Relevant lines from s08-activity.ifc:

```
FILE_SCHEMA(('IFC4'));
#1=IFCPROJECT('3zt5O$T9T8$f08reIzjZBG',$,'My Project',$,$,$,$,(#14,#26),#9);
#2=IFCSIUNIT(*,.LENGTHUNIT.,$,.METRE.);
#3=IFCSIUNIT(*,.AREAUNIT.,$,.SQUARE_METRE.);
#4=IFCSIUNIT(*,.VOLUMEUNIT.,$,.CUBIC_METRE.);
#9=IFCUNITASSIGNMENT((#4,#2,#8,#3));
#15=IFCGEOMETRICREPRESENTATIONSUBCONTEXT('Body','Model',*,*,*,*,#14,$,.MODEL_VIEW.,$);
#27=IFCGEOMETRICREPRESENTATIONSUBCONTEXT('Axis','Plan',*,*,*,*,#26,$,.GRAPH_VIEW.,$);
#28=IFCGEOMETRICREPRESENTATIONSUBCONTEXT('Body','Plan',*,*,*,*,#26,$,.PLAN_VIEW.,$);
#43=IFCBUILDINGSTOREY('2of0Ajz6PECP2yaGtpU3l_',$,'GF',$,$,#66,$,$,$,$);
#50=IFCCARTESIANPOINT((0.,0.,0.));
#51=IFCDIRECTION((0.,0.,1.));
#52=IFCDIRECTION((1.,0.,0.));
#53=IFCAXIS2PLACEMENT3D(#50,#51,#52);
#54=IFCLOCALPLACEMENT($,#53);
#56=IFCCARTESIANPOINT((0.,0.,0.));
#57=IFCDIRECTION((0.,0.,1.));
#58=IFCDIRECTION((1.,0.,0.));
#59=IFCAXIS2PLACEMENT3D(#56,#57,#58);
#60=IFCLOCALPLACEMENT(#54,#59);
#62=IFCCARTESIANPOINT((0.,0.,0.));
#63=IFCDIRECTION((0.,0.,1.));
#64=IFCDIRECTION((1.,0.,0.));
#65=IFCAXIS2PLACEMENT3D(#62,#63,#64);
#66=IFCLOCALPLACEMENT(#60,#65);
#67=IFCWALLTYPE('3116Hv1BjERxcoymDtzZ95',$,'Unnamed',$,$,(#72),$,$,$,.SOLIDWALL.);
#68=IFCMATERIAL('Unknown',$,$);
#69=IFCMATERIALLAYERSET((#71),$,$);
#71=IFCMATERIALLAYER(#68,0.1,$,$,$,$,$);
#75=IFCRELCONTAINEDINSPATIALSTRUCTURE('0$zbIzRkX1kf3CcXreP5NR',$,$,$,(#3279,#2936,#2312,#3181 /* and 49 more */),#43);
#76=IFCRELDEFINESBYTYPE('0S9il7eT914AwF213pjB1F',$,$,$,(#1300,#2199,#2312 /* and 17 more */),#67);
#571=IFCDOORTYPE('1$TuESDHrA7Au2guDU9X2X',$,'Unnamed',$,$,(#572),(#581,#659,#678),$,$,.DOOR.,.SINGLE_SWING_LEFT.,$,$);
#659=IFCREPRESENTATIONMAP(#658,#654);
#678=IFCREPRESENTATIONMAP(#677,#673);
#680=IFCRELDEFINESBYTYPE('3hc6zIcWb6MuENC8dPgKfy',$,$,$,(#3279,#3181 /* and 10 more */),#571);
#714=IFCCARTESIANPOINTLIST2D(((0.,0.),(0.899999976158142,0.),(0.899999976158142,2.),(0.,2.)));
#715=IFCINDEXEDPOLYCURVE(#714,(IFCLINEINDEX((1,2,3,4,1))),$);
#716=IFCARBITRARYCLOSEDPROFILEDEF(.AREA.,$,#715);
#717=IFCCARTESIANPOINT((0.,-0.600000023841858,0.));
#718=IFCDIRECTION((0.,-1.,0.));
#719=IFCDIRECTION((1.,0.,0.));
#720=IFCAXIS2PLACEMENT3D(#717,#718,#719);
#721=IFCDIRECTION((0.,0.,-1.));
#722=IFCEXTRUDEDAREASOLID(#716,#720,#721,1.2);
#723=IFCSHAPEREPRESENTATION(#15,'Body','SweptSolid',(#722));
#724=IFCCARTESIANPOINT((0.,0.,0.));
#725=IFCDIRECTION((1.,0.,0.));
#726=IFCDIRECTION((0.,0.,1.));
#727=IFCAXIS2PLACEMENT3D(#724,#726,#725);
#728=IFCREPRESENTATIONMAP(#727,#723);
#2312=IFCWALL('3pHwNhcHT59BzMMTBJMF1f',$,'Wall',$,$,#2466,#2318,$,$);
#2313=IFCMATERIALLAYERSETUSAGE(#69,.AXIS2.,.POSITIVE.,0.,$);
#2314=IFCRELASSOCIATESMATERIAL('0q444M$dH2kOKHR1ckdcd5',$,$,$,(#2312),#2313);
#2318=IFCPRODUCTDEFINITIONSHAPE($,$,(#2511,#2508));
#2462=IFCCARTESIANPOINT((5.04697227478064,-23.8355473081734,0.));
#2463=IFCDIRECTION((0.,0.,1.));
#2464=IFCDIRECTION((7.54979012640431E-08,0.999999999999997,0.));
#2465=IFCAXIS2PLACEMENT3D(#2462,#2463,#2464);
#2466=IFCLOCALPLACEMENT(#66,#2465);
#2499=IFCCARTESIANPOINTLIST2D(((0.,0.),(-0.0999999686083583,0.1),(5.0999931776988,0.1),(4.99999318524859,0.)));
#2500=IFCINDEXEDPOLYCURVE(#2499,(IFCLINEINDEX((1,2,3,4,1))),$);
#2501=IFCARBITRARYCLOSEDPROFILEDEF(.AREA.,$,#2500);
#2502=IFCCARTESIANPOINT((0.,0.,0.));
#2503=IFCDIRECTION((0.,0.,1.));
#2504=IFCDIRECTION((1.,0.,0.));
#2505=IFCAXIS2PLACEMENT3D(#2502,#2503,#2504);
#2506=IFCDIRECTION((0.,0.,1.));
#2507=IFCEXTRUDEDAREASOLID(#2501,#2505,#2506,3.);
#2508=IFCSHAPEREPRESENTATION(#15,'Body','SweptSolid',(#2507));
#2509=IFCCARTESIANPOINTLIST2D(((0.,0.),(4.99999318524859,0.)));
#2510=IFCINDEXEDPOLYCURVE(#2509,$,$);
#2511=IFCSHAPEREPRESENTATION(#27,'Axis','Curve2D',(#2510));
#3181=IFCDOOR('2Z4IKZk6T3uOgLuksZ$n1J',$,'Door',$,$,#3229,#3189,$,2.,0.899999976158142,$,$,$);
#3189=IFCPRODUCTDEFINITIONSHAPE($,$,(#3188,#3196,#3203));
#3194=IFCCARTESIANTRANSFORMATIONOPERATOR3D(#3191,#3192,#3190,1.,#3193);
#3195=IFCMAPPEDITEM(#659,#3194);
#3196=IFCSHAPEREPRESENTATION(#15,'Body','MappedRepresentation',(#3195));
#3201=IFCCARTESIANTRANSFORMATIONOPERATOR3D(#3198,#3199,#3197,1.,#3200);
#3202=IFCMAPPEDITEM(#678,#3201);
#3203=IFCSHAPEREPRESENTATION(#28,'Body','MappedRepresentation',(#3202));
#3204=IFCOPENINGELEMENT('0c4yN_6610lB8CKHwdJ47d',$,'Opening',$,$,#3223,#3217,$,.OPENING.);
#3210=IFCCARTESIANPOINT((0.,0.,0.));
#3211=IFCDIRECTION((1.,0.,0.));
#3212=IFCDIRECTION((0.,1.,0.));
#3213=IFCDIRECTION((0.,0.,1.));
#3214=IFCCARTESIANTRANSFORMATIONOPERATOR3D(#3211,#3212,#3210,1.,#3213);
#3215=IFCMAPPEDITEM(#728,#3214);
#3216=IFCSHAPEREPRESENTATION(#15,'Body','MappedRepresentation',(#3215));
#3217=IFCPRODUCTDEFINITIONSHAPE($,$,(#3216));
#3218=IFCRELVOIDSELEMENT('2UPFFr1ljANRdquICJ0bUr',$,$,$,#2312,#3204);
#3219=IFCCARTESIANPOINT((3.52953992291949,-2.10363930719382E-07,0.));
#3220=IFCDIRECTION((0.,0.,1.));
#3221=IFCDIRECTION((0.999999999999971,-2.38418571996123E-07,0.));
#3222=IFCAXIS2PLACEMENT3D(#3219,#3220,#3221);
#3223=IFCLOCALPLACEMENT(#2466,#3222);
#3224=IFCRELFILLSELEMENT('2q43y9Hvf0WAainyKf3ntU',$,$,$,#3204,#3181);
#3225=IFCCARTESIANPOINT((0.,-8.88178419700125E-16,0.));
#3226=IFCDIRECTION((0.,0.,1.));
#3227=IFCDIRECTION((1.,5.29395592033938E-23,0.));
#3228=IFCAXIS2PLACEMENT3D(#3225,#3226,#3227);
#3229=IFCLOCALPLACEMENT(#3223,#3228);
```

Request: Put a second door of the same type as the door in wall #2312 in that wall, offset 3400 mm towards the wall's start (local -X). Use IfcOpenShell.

```python
import ifcopenshell
import ifcopenshell.api.feature
import ifcopenshell.api.geometry
import ifcopenshell.api.root
import ifcopenshell.geom
import ifcopenshell.util.element
import ifcopenshell.util.placement
import ifcopenshell.util.shape
import ifcopenshell.util.unit

model = ifcopenshell.open("s08-activity.ifc")
unit_scale = ifcopenshell.util.unit.calculate_unit_scale(model)
settings = ifcopenshell.geom.settings()


def volume(element):
    """Net volume in cubic metres, openings subtracted."""
    shape = ifcopenshell.geom.create_shape(settings, element)
    return ifcopenshell.util.shape.get_volume(shape.geometry)


door = model.by_guid("2Z4IKZk6T3uOgLuksZ$n1J")
opening = door.FillsVoids[0].RelatingOpeningElement
wall = opening.VoidsElements[0].RelatingBuildingElement
before = volume(wall)
shift = ifcopenshell.util.placement.get_local_placement(wall.ObjectPlacement)[:3, 0] * -3.4 / unit_scale

# copy_class copies the void relationship, type, container and properties, but no geometry.
new_opening = ifcopenshell.api.root.copy_class(model, product=opening)
new_opening.Representation = ifcopenshell.util.element.copy_deep(
    model, opening.Representation, exclude=["IfcGeometricRepresentationContext", "IfcRepresentationMap"]
)
new_door = ifcopenshell.api.root.copy_class(model, product=door)
new_door.Representation = ifcopenshell.util.element.copy_deep(
    model, door.Representation, exclude=["IfcGeometricRepresentationContext", "IfcRepresentationMap"]
)
ifcopenshell.api.feature.add_filling(model, opening=new_opening, element=new_door)

for old, new in ((opening, new_opening), (door, new_door)):
    matrix = ifcopenshell.util.placement.get_local_placement(old.ObjectPlacement)
    matrix[:3, 3] += shift
    ifcopenshell.api.geometry.edit_object_placement(model, product=new, matrix=matrix, is_si=False)

after = volume(wall)

print(f"wall volume {before:.3f} -> {after:.3f} m3")

model.write("s08-activity_rev.ifc")
```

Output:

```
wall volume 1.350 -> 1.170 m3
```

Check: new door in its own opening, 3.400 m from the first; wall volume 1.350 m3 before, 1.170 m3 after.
